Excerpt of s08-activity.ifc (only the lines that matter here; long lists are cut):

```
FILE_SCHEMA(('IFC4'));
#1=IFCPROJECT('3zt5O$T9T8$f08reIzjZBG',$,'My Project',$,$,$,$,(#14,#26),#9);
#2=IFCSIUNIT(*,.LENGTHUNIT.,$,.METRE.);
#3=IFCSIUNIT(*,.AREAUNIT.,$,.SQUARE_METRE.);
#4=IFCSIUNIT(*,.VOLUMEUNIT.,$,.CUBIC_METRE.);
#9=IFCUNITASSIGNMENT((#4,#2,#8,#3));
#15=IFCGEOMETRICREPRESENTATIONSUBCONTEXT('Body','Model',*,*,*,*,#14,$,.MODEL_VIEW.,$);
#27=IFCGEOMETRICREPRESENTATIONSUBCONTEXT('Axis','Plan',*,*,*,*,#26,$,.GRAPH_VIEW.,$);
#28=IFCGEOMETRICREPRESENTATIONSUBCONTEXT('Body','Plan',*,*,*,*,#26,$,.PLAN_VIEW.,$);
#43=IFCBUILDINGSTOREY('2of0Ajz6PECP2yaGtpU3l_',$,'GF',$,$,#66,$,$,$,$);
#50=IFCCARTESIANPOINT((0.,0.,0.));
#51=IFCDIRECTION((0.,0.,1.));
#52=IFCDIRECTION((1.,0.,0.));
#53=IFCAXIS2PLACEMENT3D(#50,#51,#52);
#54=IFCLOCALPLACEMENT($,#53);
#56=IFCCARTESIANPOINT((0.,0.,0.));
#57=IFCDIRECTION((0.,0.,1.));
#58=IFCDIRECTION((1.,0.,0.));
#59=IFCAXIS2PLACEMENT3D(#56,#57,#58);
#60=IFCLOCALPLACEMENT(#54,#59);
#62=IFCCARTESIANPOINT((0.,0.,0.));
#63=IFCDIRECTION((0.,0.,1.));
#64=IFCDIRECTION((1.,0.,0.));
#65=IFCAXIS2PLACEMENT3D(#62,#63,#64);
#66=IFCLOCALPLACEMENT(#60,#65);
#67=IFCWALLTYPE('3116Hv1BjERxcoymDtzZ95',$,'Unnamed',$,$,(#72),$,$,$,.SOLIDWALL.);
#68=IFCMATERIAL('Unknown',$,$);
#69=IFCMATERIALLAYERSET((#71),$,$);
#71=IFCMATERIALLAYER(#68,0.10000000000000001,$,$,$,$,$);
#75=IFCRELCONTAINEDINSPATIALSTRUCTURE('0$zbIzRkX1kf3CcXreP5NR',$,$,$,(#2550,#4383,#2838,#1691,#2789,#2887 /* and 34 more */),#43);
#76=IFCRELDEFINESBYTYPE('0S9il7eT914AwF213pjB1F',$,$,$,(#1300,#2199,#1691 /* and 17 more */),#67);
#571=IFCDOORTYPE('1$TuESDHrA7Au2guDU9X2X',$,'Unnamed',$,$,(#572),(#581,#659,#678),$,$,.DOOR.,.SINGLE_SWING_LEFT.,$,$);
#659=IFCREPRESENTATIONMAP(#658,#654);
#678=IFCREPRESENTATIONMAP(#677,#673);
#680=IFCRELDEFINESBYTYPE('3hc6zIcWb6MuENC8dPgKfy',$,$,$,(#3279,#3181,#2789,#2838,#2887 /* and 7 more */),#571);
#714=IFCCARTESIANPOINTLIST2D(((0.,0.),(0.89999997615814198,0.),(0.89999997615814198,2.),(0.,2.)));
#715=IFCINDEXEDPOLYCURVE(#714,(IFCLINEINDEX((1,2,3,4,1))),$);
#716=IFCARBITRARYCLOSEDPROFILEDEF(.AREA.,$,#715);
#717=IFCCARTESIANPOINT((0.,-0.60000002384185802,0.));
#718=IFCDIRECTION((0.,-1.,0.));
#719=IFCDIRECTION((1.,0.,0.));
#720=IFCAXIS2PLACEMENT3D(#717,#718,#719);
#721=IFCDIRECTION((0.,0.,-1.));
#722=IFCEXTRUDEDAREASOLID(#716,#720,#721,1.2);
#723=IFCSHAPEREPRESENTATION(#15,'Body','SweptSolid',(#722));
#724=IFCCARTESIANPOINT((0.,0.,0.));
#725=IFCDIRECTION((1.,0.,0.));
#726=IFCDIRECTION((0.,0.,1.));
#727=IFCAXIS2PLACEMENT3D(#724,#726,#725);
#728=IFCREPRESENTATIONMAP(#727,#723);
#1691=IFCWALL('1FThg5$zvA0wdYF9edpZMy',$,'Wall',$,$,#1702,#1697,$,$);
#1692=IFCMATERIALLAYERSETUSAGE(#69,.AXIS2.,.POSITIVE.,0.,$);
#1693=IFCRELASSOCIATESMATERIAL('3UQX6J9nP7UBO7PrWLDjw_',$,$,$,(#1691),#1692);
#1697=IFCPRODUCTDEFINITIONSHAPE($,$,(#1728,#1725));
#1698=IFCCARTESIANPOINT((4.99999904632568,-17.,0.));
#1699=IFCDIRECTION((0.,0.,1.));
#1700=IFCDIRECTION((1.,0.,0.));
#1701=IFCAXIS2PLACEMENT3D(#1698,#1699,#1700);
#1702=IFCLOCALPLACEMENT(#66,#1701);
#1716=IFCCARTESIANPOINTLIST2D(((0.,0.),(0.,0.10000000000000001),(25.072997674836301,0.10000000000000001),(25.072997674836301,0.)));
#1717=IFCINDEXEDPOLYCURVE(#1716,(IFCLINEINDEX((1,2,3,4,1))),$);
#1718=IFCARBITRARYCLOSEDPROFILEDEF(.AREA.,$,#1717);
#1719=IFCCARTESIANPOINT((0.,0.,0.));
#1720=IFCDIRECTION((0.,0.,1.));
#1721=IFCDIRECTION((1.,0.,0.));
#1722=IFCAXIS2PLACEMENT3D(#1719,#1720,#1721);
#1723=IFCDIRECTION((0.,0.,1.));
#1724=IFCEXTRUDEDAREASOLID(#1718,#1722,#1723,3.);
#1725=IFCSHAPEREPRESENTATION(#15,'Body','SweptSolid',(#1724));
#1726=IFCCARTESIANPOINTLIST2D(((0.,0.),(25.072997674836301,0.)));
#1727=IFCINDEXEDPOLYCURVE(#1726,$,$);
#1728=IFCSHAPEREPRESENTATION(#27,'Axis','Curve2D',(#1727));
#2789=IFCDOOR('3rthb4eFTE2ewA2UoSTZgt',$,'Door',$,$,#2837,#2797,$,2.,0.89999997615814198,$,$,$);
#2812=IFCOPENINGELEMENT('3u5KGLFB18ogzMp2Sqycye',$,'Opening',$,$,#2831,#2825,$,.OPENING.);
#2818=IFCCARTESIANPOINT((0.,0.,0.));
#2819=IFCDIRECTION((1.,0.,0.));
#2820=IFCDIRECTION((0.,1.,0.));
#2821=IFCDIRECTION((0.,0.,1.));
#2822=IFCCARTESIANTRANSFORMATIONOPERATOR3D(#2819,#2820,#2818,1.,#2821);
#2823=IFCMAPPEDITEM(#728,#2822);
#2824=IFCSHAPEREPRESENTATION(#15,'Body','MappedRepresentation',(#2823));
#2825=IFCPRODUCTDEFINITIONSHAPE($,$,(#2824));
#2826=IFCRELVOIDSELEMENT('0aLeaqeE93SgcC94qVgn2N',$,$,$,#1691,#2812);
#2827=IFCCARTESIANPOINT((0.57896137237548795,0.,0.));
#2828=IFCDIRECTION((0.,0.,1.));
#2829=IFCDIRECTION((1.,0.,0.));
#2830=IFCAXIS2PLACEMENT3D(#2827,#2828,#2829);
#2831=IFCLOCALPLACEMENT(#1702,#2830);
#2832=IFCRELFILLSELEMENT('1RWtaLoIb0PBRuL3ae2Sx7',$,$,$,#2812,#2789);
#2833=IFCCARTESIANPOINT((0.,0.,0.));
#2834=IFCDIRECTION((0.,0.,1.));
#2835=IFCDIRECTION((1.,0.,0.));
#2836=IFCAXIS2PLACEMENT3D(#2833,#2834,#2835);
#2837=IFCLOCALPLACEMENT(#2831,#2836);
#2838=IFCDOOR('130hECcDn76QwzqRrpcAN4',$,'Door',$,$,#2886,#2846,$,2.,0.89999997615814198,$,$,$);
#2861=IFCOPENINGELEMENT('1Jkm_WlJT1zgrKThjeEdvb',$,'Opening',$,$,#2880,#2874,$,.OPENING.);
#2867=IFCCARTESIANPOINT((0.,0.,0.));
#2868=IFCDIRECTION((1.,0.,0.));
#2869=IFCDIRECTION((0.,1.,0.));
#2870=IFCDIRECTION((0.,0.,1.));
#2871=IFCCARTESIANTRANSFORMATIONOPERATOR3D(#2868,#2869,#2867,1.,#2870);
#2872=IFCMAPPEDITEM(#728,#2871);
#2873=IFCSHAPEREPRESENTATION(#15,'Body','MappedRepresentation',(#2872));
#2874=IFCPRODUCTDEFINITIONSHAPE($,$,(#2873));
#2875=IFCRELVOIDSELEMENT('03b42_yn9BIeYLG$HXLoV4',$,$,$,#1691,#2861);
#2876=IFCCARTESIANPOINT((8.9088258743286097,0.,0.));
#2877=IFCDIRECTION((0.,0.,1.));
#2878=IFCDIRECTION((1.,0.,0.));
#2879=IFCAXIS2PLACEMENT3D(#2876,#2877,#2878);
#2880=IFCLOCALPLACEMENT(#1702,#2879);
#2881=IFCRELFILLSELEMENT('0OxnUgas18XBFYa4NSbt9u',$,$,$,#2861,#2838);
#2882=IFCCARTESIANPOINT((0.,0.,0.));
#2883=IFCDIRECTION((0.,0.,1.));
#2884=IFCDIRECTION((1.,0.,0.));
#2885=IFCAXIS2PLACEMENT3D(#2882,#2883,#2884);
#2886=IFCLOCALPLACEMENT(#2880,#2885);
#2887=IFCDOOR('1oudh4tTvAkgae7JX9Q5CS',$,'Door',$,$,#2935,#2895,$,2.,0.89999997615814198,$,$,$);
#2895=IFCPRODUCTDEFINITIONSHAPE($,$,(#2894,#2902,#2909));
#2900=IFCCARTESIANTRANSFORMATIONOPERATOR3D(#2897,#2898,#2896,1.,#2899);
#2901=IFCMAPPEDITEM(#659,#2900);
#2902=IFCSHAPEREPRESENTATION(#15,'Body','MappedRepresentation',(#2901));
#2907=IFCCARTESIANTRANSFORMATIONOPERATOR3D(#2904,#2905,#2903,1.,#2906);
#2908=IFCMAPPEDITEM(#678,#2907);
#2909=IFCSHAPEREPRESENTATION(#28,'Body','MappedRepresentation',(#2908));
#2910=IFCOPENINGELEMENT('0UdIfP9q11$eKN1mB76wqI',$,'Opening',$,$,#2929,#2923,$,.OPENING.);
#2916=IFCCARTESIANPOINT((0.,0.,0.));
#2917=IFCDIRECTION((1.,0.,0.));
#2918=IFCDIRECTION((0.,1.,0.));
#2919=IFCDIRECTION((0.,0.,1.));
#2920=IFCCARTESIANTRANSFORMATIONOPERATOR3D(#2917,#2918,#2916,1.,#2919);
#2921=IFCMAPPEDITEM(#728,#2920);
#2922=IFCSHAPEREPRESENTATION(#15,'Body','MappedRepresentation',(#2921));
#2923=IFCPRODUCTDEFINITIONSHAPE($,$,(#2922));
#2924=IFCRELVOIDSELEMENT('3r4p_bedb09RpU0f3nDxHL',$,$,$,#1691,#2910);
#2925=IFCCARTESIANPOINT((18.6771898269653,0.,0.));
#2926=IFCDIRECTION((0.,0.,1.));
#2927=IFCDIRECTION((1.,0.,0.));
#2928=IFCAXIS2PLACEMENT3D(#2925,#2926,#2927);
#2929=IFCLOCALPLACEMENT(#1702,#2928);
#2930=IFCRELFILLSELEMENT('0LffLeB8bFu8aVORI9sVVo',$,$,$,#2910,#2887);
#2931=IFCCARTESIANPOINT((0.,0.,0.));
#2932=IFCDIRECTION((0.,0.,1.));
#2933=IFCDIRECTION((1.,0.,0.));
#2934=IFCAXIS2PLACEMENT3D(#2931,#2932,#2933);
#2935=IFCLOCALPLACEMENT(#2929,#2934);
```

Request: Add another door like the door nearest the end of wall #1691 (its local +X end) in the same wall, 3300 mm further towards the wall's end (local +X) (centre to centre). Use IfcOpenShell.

```python
import ifcopenshell
import ifcopenshell.api.feature
import ifcopenshell.api.geometry
import ifcopenshell.api.root
import ifcopenshell.geom
import ifcopenshell.util.element
import ifcopenshell.util.placement
import ifcopenshell.util.shape

model = ifcopenshell.open("s08-activity.ifc")
settings = ifcopenshell.geom.settings()


def volume(element):
    """Net volume in cubic metres, openings subtracted."""
    shape = ifcopenshell.geom.create_shape(settings, element)
    return ifcopenshell.util.shape.get_volume(shape.geometry)


door = model.by_guid("1oudh4tTvAkgae7JX9Q5CS")
opening = door.FillsVoids[0].RelatingOpeningElement
wall = opening.VoidsElements[0].RelatingBuildingElement
before = volume(wall)
shift = ifcopenshell.util.placement.get_local_placement(wall.ObjectPlacement)[:3, 0] * 3.3

# copy_class copies the void relationship, type, container and properties, but no geometry.
new_opening = ifcopenshell.api.root.copy_class(model, product=opening)
new_opening.Representation = ifcopenshell.util.element.copy_deep(
    model, opening.Representation, exclude=["IfcGeometricRepresentationContext", "IfcRepresentationMap"]
)
new_door = ifcopenshell.api.root.copy_class(model, product=door)
new_door.Representation = ifcopenshell.util.element.copy_deep(
    model, door.Representation, exclude=["IfcGeometricRepresentationContext", "IfcRepresentationMap"]
)
ifcopenshell.api.feature.add_filling(model, opening=new_opening, element=new_door)

for old, new in ((opening, new_opening), (door, new_door)):
    matrix = ifcopenshell.util.placement.get_local_placement(old.ObjectPlacement)
    matrix[:3, 3] += shift
    ifcopenshell.api.geometry.edit_object_placement(model, product=new, matrix=matrix, is_si=False)

after = volume(wall)

print(f"wall volume {before:.3f} -> {after:.3f} m3")

model.write("s08-activity-out.ifc")
```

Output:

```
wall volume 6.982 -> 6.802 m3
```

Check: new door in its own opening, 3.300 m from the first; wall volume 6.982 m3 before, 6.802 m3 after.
